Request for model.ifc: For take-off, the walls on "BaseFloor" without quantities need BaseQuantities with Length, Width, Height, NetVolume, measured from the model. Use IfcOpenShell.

First a look at what the model holds.

```python
import ifcopenshell
import ifcopenshell.util.element
import ifcopenshell.util.unit

model = ifcopenshell.open("model.ifc")
print(model.schema)
for unit_type in ("LENGTHUNIT", "AREAUNIT", "VOLUMEUNIT"):
    print(unit_type, ifcopenshell.util.unit.calculate_unit_scale(model, unit_type))
storey = next(s for s in model.by_type("IfcBuildingStorey") if s.Name == "BaseFloor")
walls = [e for e in ifcopenshell.util.element.get_decomposition(storey) if e.is_a("IfcWall")]
for e in sorted(walls, key=lambda e: e.id()):
    print(e.id(), e.is_a(), e.Name, list(ifcopenshell.util.element.get_psets(e, qtos_only=True)), sep=" | ")
```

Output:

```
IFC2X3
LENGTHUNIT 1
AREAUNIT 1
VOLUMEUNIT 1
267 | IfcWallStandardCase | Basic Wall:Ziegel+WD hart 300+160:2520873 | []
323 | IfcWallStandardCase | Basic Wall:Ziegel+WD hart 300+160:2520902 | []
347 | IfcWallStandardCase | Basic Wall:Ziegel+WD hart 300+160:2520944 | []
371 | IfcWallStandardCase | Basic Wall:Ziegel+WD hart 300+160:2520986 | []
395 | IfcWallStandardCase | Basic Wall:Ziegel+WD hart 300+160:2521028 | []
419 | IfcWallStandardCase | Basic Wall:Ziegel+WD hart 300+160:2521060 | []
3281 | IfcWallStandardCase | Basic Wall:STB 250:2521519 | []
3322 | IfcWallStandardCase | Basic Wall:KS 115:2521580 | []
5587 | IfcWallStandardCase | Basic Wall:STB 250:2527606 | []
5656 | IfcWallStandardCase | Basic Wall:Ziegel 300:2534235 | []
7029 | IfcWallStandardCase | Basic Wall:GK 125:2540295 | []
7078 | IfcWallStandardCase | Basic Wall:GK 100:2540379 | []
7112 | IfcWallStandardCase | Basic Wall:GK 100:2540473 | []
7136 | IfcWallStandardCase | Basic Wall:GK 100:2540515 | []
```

```python
import ifcopenshell
import ifcopenshell.api.pset
import ifcopenshell.geom
import ifcopenshell.util.element
import ifcopenshell.util.shape
import ifcopenshell.util.unit

model = ifcopenshell.open("model.ifc")
unit_scale = ifcopenshell.util.unit.calculate_unit_scale(model)
volume_scale = ifcopenshell.util.unit.calculate_unit_scale(model, "VOLUMEUNIT")
settings = ifcopenshell.geom.settings()

storey = next(s for s in model.by_type("IfcBuildingStorey") if s.Name == "BaseFloor")
walls = [e for e in ifcopenshell.util.element.get_decomposition(storey) if e.is_a("IfcWall")]

for e in sorted(walls, key=lambda e: e.id()):
    if ifcopenshell.util.element.get_psets(e, qtos_only=True, should_inherit=False):
        continue
    # Geometry comes back in metres, in the element's own axes.
    shape = ifcopenshell.geom.create_shape(settings, e)
    values = {
        "Length": ifcopenshell.util.shape.get_x(shape.geometry) / unit_scale,
        "Width": ifcopenshell.util.shape.get_y(shape.geometry) / unit_scale,
        "Height": ifcopenshell.util.shape.get_z(shape.geometry) / unit_scale,
        "NetVolume": ifcopenshell.util.shape.get_volume(shape.geometry) / volume_scale,
    }
    qto = ifcopenshell.api.pset.add_qto(model, product=e, name="BaseQuantities")
    ifcopenshell.api.pset.edit_qto(model, qto=qto, properties=values)
    print(e.id(), {k: round(v, 3) for k, v in values.items()})

model.write("model_updated.ifc")
```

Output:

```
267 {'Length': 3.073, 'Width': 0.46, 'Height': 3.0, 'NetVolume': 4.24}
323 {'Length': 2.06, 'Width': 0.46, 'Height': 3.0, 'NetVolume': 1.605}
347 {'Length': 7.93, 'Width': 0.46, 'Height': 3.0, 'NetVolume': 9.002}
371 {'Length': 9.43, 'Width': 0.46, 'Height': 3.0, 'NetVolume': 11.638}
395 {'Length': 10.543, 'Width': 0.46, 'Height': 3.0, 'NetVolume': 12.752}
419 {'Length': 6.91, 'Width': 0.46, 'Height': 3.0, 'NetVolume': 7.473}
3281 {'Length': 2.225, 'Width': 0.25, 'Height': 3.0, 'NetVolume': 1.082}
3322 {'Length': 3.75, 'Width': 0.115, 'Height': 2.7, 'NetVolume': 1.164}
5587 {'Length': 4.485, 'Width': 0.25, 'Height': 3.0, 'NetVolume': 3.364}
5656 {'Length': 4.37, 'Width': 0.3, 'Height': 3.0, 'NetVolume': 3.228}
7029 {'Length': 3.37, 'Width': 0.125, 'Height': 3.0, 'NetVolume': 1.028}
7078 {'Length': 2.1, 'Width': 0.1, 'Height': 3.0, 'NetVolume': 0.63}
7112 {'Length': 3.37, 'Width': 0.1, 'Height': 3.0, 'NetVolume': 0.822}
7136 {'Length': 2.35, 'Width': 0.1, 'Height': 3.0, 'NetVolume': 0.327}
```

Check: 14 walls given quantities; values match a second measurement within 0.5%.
